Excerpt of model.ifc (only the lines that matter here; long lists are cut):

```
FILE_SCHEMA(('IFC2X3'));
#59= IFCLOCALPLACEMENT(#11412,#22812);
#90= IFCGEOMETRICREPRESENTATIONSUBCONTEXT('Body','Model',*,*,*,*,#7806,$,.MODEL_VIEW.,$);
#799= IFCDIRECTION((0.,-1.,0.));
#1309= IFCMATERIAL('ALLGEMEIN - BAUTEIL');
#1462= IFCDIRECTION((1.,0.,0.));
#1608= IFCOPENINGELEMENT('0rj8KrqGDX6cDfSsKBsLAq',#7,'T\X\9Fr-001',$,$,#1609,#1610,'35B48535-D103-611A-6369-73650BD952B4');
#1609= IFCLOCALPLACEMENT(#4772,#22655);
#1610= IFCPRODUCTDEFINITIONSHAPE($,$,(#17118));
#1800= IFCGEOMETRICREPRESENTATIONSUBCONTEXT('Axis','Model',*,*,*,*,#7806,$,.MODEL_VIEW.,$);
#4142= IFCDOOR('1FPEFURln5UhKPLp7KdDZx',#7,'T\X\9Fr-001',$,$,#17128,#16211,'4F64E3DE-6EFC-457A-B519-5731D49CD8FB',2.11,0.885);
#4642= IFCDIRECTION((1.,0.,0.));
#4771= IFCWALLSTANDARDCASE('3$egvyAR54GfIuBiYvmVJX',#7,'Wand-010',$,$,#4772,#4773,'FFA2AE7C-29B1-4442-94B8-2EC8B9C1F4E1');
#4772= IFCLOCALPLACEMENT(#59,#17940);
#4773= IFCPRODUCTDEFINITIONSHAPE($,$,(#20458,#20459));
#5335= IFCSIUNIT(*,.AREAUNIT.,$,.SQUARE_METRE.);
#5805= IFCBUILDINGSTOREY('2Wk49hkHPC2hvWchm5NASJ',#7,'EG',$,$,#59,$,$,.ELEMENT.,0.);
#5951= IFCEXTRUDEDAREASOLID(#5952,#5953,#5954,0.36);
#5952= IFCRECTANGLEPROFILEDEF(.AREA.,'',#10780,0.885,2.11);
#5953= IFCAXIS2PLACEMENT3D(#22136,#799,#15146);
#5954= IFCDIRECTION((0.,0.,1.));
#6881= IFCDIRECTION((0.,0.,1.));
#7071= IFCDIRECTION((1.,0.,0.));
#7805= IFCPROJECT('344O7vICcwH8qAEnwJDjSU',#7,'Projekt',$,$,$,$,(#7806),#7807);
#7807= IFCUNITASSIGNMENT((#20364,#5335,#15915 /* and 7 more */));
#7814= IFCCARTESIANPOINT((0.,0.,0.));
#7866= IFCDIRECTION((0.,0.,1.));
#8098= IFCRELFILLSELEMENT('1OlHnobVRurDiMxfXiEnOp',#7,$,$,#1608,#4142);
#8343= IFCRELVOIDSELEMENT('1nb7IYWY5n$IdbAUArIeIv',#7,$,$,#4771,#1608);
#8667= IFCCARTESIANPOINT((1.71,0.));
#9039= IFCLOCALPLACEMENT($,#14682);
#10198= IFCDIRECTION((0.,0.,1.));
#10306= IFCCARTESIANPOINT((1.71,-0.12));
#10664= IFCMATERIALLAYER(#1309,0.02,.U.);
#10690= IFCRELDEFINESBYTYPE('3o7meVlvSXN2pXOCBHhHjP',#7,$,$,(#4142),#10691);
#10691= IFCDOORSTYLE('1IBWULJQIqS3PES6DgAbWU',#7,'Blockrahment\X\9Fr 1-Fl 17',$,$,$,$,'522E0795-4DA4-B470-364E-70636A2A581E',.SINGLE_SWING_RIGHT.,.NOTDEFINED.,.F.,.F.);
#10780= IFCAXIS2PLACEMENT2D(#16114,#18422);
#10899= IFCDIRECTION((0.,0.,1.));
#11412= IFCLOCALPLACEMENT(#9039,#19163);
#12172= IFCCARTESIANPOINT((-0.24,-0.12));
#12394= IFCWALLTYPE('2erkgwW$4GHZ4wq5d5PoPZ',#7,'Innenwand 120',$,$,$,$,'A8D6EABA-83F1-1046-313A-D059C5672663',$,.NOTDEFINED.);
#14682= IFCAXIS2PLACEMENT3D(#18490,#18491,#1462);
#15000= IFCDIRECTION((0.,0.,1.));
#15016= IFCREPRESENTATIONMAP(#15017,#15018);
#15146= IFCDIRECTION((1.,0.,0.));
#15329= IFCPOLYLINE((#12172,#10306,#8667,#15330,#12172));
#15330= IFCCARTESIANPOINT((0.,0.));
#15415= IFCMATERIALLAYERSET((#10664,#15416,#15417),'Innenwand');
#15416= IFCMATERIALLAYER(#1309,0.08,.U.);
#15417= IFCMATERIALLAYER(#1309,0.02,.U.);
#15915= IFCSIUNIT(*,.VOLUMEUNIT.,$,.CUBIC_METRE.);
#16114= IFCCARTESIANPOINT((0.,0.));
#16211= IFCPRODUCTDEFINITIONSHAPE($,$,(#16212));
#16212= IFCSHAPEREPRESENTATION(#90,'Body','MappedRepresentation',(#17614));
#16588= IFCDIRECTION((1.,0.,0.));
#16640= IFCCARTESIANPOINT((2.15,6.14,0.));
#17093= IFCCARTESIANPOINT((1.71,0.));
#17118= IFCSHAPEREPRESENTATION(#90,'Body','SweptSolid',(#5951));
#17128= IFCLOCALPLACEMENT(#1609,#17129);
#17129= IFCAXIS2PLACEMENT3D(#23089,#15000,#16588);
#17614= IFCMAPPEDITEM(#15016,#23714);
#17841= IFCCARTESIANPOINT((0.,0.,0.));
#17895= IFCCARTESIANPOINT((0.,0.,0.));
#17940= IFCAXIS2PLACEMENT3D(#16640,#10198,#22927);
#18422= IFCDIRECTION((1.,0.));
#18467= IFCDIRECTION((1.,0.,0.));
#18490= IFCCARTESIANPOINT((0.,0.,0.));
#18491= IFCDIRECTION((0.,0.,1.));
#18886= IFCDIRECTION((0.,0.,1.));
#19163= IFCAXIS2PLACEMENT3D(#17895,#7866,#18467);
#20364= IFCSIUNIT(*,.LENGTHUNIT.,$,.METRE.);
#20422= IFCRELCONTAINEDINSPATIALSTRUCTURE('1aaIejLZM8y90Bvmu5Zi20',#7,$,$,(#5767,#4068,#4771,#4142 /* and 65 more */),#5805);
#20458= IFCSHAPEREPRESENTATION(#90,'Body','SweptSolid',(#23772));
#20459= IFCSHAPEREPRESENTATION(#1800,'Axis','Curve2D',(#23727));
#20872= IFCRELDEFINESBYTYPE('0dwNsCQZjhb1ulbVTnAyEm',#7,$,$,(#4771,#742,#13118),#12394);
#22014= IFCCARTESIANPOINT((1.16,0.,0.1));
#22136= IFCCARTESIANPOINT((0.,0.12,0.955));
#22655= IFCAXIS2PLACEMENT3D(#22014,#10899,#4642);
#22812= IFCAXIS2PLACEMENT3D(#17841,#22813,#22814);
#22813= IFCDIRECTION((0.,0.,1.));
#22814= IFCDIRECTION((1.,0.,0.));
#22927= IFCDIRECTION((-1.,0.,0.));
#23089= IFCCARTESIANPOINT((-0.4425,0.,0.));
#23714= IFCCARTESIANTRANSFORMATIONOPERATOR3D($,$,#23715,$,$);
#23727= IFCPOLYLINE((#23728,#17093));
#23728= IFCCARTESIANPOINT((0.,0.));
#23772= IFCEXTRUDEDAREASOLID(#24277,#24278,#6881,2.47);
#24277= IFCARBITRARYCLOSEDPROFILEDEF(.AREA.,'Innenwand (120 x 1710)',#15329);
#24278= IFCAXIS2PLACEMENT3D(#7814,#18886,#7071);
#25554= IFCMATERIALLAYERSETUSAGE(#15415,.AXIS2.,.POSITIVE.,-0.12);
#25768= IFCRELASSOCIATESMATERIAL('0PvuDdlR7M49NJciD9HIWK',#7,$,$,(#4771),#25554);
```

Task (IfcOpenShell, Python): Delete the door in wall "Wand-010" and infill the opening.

```python
import ifcopenshell
import ifcopenshell.api.feature
import ifcopenshell.api.root
import ifcopenshell.geom
import ifcopenshell.util.shape

model = ifcopenshell.open("model.ifc")
settings = ifcopenshell.geom.settings()


def volume(element):
    """Net volume in cubic metres, openings subtracted."""
    shape = ifcopenshell.geom.create_shape(settings, element)
    return ifcopenshell.util.shape.get_volume(shape.geometry)


door = model.by_guid("1FPEFURln5UhKPLp7KdDZx")
opening = door.FillsVoids[0].RelatingOpeningElement
wall = opening.VoidsElements[0].RelatingBuildingElement
before = volume(wall)

ifcopenshell.api.root.remove_product(model, product=door)
ifcopenshell.api.feature.remove_feature(model, feature=opening)

after = volume(wall)

print(f"wall volume {before:.3f} -> {after:.3f} m3")

model.write("model_edited.ifc")
```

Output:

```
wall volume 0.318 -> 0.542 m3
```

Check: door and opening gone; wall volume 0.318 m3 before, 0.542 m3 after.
